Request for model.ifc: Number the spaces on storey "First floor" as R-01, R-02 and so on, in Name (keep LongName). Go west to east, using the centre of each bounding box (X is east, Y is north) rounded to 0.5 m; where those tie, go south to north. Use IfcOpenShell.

First a look at what the model holds.

```python
import ifcopenshell
import ifcopenshell.util.element
import ifcopenshell.util.placement

model = ifcopenshell.open("model.ifc")
print(model.schema)
storey = next(s for s in model.by_type("IfcBuildingStorey") if s.Name == "First floor")
spaces = [e for e in ifcopenshell.util.element.get_decomposition(storey) if e.is_a("IfcSpace")]
for e in sorted(spaces, key=lambda e: e.id()):
    origin = ifcopenshell.util.placement.get_local_placement(e.ObjectPlacement)[:3, 3]
    print(e.id(), e.Name, e.LongName, origin.round(2) + 0.0, sep=" | ")
```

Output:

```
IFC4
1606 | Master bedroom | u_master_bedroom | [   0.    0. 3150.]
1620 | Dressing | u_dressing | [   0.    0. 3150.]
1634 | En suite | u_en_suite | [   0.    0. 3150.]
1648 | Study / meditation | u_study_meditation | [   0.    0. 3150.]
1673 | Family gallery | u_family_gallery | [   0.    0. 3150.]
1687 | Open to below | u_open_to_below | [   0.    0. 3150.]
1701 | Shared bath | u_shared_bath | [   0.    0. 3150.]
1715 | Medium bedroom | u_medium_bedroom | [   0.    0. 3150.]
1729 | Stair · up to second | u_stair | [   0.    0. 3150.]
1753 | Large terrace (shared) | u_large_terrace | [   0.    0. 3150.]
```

```python
import ifcopenshell
import ifcopenshell.geom
import ifcopenshell.util.element
import ifcopenshell.util.shape

model = ifcopenshell.open("model.ifc")
settings = ifcopenshell.geom.settings()
settings.set("use-world-coords", True)


def centre(element):
    shape = ifcopenshell.geom.create_shape(settings, element)
    return ifcopenshell.util.shape.get_bbox_centroid(shape.geometry)


storey = next(s for s in model.by_type("IfcBuildingStorey") if s.Name == "First floor")
spaces = [e for e in ifcopenshell.util.element.get_decomposition(storey) if e.is_a("IfcSpace")]

# Insertion points can sit at a corner or the storey origin, so sort by the geometry (in metres).
centres = {e: centre(e) for e in spaces}
spaces.sort(key=lambda e: (round(centres[e][0] / 0.5), centres[e][1]))

for i, e in enumerate(spaces, start=1):
    number = f"R-{i:02d}"
    e.Name = number
    print(e.id(), number)

model.write("model_edited.ifc")
```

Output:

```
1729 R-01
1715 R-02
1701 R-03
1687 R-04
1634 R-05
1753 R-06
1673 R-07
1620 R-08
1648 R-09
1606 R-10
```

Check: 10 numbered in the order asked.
